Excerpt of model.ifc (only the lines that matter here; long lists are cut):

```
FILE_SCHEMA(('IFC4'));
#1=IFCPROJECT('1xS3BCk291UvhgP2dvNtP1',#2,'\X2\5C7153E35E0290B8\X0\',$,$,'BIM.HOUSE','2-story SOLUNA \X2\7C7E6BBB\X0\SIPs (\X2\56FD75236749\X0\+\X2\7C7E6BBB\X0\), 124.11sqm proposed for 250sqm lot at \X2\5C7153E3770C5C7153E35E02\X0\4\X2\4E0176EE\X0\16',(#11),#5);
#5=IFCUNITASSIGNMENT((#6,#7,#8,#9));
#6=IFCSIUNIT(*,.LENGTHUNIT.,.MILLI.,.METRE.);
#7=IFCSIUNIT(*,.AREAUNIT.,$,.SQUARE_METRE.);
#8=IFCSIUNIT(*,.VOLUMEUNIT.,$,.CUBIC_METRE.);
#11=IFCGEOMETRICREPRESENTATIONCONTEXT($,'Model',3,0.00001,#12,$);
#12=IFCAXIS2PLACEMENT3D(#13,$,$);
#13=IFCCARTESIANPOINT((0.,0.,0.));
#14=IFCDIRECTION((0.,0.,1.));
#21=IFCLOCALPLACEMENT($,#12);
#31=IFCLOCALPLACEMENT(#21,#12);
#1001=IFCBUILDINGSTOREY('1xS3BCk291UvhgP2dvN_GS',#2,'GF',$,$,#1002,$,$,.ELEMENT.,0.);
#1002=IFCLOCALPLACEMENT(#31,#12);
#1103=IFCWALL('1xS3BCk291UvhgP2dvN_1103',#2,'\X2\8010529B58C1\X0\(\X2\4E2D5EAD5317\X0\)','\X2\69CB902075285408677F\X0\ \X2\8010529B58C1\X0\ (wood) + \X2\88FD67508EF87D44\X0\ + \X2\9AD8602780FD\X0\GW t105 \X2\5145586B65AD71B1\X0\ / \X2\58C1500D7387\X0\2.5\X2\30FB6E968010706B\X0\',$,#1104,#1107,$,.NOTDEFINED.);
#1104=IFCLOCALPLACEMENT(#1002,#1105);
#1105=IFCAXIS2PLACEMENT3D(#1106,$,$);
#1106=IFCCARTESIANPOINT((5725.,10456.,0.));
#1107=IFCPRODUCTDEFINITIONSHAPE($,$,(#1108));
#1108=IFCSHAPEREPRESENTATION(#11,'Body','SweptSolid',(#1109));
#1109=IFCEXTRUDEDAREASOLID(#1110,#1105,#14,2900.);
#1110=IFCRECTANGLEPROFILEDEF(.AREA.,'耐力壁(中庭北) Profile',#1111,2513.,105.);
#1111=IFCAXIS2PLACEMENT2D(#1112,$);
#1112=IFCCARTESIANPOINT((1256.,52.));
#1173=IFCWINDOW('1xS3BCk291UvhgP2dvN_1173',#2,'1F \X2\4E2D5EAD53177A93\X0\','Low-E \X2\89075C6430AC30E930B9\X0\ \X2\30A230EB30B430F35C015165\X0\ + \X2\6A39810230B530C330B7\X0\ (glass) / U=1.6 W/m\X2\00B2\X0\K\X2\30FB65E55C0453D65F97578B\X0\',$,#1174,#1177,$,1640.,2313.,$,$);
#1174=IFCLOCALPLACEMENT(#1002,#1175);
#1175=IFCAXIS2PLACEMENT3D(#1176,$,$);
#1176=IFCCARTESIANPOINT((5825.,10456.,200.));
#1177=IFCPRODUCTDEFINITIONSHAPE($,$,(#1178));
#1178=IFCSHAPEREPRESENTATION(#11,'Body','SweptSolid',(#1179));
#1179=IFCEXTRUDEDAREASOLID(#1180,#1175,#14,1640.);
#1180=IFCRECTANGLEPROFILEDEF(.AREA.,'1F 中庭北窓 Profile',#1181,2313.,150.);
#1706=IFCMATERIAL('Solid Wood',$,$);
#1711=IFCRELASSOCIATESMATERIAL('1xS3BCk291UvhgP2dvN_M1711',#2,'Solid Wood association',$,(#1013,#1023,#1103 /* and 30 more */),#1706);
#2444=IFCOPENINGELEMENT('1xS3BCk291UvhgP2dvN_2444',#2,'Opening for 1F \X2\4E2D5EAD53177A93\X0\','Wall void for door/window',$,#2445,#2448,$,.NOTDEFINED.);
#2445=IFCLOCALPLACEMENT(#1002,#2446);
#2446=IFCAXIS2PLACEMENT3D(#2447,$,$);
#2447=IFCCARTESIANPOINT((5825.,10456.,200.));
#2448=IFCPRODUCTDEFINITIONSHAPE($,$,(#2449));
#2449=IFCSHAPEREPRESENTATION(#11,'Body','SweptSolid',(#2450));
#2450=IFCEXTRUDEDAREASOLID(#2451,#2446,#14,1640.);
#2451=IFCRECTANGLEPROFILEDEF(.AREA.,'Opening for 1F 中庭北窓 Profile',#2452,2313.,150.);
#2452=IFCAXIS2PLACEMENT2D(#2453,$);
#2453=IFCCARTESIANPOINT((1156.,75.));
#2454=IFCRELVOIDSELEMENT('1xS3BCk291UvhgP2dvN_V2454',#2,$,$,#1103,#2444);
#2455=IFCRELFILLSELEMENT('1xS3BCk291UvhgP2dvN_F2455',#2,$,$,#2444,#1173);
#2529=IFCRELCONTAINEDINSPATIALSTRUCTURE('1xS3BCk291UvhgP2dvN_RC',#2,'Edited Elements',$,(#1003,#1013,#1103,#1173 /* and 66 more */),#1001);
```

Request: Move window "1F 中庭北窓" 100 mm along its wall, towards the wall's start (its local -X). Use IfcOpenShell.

```python
import ifcopenshell
import ifcopenshell.api.geometry
import ifcopenshell.util.placement

model = ifcopenshell.open("model.ifc")

window = model.by_id(1173)
opening = window.FillsVoids[0].RelatingOpeningElement
wall = opening.VoidsElements[0].RelatingBuildingElement

wall_matrix = ifcopenshell.util.placement.get_local_placement(wall.ObjectPlacement)
shift = wall_matrix[:3, 0] * -100.0
before = ifcopenshell.util.placement.get_local_placement(window.ObjectPlacement)[:3, 3].copy()

# The window is not placed relative to its opening, so move both.
for product in (opening, window):
    matrix = ifcopenshell.util.placement.get_local_placement(product.ObjectPlacement)
    matrix[:3, 3] += shift
    ifcopenshell.api.geometry.edit_object_placement(model, product=product, matrix=matrix, is_si=False)

after = ifcopenshell.util.placement.get_local_placement(window.ObjectPlacement)[:3, 3]
print("window moved by", (after - before).round(3) + 0.0)

model.write("model_edited.ifc")
```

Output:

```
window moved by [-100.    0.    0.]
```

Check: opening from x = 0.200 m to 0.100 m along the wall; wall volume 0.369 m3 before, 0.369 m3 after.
